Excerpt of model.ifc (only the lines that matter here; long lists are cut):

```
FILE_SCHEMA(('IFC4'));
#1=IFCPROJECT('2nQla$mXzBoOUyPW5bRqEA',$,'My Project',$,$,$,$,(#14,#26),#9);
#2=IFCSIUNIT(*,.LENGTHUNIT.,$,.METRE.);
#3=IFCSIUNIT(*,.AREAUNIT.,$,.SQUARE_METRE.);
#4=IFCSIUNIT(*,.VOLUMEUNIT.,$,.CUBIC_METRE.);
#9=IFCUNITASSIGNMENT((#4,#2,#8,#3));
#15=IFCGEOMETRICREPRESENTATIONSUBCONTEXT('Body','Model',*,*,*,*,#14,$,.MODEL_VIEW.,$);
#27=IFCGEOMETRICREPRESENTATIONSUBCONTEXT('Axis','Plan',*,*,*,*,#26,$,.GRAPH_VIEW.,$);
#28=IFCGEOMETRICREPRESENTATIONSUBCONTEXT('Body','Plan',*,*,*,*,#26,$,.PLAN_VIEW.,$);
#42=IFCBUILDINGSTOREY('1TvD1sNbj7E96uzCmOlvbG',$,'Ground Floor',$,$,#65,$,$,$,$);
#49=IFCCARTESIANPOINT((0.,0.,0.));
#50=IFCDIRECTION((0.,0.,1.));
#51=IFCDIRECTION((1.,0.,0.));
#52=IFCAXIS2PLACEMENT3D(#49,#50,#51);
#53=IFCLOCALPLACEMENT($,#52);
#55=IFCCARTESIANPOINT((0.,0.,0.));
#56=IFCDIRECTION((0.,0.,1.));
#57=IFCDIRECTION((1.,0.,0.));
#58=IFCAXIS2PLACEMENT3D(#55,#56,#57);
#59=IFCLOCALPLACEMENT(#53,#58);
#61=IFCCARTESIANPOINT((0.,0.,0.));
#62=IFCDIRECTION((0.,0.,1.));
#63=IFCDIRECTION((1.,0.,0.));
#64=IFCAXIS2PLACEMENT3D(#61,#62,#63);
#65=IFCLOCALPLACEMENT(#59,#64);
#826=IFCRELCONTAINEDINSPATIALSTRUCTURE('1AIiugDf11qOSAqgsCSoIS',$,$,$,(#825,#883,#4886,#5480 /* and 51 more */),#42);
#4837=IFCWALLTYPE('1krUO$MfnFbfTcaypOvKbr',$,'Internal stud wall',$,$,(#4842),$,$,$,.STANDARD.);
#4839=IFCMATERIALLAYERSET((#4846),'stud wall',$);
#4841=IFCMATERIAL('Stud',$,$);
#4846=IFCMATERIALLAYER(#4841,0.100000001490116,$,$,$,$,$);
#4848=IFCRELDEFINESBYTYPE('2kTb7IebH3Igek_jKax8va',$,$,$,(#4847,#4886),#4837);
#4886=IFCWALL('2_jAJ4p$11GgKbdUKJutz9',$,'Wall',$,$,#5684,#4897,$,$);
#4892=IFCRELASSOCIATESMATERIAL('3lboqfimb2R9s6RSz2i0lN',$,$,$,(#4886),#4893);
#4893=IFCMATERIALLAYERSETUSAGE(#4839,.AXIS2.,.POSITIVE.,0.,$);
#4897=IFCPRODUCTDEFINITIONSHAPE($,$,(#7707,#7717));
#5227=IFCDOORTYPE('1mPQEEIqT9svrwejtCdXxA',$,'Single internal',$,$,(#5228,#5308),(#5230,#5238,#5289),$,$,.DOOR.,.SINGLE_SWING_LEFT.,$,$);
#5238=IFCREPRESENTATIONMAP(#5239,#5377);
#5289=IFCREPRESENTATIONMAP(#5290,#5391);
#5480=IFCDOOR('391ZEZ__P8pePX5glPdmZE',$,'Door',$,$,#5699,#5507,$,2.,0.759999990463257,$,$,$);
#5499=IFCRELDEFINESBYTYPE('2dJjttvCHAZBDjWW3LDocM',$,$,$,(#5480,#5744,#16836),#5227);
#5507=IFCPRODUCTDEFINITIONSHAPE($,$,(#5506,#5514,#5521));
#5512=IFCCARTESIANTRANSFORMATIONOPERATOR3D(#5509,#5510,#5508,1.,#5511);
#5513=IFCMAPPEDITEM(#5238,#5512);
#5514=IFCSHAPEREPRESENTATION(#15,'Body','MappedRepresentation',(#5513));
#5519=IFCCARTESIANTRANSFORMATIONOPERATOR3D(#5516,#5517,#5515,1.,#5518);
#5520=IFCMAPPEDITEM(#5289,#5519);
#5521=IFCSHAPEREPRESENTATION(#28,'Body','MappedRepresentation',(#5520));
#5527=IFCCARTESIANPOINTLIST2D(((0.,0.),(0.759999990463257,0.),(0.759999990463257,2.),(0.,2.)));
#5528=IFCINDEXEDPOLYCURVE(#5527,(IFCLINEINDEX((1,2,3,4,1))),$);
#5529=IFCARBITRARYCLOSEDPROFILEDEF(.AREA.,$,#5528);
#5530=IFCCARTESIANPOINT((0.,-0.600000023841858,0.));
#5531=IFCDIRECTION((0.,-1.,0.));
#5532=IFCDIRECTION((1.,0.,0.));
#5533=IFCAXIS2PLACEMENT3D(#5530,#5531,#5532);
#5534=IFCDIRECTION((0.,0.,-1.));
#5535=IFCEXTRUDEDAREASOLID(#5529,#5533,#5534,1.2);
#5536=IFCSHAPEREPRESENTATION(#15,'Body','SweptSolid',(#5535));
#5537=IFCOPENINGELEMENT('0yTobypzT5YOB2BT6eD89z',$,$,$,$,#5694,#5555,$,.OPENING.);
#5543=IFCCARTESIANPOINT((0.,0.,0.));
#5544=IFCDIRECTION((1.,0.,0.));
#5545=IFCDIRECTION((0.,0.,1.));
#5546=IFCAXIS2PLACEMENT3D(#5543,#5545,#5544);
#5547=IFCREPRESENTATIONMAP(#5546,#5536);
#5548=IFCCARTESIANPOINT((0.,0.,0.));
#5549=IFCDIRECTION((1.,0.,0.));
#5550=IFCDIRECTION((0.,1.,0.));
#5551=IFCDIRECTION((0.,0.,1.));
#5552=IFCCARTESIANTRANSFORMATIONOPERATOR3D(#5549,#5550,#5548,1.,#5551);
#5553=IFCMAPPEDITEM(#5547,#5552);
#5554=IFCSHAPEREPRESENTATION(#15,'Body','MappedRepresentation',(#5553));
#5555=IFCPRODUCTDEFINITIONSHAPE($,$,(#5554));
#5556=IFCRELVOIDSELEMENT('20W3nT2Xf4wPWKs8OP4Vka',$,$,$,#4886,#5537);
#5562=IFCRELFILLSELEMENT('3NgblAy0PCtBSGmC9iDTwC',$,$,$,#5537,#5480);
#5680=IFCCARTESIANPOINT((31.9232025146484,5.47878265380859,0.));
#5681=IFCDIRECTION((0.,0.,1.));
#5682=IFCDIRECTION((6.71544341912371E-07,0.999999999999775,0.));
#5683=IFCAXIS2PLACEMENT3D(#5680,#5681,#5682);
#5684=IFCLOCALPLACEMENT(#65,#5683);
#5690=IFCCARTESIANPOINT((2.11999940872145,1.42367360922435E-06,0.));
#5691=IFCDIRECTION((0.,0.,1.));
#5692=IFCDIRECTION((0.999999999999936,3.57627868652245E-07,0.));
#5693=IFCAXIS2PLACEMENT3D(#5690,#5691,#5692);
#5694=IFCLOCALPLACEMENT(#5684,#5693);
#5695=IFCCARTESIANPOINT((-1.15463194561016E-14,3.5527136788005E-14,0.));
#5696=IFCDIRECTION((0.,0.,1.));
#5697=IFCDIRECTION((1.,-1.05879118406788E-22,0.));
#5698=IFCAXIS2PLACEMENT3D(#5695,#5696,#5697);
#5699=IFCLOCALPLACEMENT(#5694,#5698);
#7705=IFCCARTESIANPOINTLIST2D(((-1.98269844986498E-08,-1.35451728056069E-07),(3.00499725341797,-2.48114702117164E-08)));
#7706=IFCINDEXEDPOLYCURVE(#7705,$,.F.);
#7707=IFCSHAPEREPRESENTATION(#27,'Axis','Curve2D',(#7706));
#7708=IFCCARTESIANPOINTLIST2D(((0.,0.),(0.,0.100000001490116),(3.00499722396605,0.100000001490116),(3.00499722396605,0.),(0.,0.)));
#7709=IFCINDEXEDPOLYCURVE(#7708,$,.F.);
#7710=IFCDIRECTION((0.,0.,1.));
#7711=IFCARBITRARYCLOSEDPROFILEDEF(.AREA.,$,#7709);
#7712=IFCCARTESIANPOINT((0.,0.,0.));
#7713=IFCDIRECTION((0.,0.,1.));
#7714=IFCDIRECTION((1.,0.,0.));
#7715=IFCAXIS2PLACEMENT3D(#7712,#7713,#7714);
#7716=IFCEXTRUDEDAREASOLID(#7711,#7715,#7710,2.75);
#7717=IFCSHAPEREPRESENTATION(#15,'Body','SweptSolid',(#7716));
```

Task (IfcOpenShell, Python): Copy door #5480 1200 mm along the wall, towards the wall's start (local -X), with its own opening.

```python
import ifcopenshell
import ifcopenshell.api.feature
import ifcopenshell.api.geometry
import ifcopenshell.api.root
import ifcopenshell.geom
import ifcopenshell.util.element
import ifcopenshell.util.placement
import ifcopenshell.util.shape

model = ifcopenshell.open("model.ifc")
settings = ifcopenshell.geom.settings()


def volume(element):
    """Net volume in cubic metres, openings subtracted."""
    shape = ifcopenshell.geom.create_shape(settings, element)
    return ifcopenshell.util.shape.get_volume(shape.geometry)


door = model.by_guid("391ZEZ__P8pePX5glPdmZE")
opening = door.FillsVoids[0].RelatingOpeningElement
wall = opening.VoidsElements[0].RelatingBuildingElement
before = volume(wall)
shift = ifcopenshell.util.placement.get_local_placement(wall.ObjectPlacement)[:3, 0] * -1.2

# copy_class copies the void relationship, type, container and properties, but no geometry.
new_opening = ifcopenshell.api.root.copy_class(model, product=opening)
new_opening.Representation = ifcopenshell.util.element.copy_deep(
    model, opening.Representation, exclude=["IfcGeometricRepresentationContext", "IfcRepresentationMap"]
)
new_door = ifcopenshell.api.root.copy_class(model, product=door)
new_door.Representation = ifcopenshell.util.element.copy_deep(
    model, door.Representation, exclude=["IfcGeometricRepresentationContext", "IfcRepresentationMap"]
)
ifcopenshell.api.feature.add_filling(model, opening=new_opening, element=new_door)

for old, new in ((opening, new_opening), (door, new_door)):
    matrix = ifcopenshell.util.placement.get_local_placement(old.ObjectPlacement)
    matrix[:3, 3] += shift
    ifcopenshell.api.geometry.edit_object_placement(model, product=new, matrix=matrix, is_si=False)

after = volume(wall)

print(f"wall volume {before:.3f} -> {after:.3f} m3")

model.write("model_v2.ifc")
```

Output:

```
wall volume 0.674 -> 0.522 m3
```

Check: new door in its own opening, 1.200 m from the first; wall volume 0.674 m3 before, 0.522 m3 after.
